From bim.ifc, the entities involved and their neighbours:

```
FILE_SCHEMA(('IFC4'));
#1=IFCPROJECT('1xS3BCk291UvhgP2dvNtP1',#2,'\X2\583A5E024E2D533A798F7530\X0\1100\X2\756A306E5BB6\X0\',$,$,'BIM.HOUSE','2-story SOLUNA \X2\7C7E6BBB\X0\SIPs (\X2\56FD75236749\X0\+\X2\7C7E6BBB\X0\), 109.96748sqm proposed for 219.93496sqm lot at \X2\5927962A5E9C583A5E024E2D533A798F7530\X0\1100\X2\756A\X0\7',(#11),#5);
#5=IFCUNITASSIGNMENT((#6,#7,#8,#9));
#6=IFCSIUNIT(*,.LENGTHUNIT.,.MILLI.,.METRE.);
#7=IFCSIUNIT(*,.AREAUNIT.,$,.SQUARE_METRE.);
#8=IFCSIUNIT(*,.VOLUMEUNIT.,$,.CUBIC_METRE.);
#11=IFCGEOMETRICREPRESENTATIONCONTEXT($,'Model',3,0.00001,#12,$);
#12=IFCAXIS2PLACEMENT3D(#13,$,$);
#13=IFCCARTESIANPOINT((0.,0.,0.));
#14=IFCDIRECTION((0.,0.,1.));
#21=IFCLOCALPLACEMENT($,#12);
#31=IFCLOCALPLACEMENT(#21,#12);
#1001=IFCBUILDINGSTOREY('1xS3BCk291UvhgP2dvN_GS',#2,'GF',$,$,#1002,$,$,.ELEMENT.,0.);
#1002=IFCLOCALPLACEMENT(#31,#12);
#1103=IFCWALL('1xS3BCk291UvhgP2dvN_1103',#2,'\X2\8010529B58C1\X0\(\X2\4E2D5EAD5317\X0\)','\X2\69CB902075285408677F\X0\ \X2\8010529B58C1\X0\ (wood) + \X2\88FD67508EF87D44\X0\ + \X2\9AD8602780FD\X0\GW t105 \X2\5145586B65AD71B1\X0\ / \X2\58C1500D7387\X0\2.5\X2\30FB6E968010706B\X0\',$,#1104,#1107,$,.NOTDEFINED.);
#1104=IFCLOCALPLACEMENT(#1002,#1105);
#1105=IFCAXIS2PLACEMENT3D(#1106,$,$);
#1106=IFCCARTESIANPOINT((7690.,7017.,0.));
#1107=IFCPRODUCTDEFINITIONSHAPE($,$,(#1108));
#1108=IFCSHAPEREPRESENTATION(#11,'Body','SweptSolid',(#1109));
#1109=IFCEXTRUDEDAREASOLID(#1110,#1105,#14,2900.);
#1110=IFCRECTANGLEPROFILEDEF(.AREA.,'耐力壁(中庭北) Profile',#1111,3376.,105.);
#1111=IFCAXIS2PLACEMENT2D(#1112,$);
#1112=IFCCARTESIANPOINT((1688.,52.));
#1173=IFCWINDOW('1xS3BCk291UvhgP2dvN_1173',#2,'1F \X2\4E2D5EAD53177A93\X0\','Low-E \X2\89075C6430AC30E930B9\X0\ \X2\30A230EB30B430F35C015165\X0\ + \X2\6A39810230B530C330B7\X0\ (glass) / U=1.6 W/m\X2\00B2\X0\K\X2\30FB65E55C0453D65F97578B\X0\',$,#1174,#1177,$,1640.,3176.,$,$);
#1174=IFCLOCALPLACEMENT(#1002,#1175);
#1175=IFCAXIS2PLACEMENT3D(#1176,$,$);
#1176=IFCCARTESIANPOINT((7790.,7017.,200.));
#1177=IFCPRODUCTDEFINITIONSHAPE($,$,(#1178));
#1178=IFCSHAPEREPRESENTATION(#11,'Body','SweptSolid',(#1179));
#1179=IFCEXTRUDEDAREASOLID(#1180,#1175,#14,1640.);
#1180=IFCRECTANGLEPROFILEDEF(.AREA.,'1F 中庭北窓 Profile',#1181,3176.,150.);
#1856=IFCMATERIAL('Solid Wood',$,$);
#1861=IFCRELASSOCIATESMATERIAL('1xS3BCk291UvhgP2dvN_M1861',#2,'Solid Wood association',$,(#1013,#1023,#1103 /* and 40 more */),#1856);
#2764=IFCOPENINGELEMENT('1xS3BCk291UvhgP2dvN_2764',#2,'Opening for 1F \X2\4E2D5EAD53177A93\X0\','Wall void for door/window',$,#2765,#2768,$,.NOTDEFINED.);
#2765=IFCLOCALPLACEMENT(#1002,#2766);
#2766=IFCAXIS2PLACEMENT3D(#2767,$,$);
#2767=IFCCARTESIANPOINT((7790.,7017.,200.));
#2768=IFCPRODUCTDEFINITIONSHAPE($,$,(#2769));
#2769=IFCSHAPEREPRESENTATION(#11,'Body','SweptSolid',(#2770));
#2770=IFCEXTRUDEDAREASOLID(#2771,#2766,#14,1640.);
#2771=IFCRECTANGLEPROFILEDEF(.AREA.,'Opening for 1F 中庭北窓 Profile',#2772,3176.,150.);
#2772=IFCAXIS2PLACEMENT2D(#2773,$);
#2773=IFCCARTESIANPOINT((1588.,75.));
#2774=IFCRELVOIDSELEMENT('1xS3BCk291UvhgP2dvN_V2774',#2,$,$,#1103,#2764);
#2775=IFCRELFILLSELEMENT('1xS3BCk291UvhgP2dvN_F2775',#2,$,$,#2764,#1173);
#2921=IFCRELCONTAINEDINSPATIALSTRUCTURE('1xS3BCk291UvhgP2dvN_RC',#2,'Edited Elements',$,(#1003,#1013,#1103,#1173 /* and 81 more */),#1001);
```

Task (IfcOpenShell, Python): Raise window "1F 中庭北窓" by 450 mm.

```python
import numpy as np
import ifcopenshell
import ifcopenshell.api.geometry
import ifcopenshell.util.placement
import ifcopenshell.util.unit

model = ifcopenshell.open("bim.ifc")
unit_scale = ifcopenshell.util.unit.calculate_unit_scale(model)

window = model.by_id(1173)
opening = window.FillsVoids[0].RelatingOpeningElement
dz = 0.45 / unit_scale

shift = np.array([0.0, 0.0, dz])
# The window is not placed relative to its opening, so move both.
for product in (opening, window):
    matrix = ifcopenshell.util.placement.get_local_placement(product.ObjectPlacement)
    matrix[:3, 3] += shift
    ifcopenshell.api.geometry.edit_object_placement(model, product=product, matrix=matrix, is_si=False)

print(f"moved by {dz * unit_scale:+.3f} m")

model.write("bim_rev.ifc")
```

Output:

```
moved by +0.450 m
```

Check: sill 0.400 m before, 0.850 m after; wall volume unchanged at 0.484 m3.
